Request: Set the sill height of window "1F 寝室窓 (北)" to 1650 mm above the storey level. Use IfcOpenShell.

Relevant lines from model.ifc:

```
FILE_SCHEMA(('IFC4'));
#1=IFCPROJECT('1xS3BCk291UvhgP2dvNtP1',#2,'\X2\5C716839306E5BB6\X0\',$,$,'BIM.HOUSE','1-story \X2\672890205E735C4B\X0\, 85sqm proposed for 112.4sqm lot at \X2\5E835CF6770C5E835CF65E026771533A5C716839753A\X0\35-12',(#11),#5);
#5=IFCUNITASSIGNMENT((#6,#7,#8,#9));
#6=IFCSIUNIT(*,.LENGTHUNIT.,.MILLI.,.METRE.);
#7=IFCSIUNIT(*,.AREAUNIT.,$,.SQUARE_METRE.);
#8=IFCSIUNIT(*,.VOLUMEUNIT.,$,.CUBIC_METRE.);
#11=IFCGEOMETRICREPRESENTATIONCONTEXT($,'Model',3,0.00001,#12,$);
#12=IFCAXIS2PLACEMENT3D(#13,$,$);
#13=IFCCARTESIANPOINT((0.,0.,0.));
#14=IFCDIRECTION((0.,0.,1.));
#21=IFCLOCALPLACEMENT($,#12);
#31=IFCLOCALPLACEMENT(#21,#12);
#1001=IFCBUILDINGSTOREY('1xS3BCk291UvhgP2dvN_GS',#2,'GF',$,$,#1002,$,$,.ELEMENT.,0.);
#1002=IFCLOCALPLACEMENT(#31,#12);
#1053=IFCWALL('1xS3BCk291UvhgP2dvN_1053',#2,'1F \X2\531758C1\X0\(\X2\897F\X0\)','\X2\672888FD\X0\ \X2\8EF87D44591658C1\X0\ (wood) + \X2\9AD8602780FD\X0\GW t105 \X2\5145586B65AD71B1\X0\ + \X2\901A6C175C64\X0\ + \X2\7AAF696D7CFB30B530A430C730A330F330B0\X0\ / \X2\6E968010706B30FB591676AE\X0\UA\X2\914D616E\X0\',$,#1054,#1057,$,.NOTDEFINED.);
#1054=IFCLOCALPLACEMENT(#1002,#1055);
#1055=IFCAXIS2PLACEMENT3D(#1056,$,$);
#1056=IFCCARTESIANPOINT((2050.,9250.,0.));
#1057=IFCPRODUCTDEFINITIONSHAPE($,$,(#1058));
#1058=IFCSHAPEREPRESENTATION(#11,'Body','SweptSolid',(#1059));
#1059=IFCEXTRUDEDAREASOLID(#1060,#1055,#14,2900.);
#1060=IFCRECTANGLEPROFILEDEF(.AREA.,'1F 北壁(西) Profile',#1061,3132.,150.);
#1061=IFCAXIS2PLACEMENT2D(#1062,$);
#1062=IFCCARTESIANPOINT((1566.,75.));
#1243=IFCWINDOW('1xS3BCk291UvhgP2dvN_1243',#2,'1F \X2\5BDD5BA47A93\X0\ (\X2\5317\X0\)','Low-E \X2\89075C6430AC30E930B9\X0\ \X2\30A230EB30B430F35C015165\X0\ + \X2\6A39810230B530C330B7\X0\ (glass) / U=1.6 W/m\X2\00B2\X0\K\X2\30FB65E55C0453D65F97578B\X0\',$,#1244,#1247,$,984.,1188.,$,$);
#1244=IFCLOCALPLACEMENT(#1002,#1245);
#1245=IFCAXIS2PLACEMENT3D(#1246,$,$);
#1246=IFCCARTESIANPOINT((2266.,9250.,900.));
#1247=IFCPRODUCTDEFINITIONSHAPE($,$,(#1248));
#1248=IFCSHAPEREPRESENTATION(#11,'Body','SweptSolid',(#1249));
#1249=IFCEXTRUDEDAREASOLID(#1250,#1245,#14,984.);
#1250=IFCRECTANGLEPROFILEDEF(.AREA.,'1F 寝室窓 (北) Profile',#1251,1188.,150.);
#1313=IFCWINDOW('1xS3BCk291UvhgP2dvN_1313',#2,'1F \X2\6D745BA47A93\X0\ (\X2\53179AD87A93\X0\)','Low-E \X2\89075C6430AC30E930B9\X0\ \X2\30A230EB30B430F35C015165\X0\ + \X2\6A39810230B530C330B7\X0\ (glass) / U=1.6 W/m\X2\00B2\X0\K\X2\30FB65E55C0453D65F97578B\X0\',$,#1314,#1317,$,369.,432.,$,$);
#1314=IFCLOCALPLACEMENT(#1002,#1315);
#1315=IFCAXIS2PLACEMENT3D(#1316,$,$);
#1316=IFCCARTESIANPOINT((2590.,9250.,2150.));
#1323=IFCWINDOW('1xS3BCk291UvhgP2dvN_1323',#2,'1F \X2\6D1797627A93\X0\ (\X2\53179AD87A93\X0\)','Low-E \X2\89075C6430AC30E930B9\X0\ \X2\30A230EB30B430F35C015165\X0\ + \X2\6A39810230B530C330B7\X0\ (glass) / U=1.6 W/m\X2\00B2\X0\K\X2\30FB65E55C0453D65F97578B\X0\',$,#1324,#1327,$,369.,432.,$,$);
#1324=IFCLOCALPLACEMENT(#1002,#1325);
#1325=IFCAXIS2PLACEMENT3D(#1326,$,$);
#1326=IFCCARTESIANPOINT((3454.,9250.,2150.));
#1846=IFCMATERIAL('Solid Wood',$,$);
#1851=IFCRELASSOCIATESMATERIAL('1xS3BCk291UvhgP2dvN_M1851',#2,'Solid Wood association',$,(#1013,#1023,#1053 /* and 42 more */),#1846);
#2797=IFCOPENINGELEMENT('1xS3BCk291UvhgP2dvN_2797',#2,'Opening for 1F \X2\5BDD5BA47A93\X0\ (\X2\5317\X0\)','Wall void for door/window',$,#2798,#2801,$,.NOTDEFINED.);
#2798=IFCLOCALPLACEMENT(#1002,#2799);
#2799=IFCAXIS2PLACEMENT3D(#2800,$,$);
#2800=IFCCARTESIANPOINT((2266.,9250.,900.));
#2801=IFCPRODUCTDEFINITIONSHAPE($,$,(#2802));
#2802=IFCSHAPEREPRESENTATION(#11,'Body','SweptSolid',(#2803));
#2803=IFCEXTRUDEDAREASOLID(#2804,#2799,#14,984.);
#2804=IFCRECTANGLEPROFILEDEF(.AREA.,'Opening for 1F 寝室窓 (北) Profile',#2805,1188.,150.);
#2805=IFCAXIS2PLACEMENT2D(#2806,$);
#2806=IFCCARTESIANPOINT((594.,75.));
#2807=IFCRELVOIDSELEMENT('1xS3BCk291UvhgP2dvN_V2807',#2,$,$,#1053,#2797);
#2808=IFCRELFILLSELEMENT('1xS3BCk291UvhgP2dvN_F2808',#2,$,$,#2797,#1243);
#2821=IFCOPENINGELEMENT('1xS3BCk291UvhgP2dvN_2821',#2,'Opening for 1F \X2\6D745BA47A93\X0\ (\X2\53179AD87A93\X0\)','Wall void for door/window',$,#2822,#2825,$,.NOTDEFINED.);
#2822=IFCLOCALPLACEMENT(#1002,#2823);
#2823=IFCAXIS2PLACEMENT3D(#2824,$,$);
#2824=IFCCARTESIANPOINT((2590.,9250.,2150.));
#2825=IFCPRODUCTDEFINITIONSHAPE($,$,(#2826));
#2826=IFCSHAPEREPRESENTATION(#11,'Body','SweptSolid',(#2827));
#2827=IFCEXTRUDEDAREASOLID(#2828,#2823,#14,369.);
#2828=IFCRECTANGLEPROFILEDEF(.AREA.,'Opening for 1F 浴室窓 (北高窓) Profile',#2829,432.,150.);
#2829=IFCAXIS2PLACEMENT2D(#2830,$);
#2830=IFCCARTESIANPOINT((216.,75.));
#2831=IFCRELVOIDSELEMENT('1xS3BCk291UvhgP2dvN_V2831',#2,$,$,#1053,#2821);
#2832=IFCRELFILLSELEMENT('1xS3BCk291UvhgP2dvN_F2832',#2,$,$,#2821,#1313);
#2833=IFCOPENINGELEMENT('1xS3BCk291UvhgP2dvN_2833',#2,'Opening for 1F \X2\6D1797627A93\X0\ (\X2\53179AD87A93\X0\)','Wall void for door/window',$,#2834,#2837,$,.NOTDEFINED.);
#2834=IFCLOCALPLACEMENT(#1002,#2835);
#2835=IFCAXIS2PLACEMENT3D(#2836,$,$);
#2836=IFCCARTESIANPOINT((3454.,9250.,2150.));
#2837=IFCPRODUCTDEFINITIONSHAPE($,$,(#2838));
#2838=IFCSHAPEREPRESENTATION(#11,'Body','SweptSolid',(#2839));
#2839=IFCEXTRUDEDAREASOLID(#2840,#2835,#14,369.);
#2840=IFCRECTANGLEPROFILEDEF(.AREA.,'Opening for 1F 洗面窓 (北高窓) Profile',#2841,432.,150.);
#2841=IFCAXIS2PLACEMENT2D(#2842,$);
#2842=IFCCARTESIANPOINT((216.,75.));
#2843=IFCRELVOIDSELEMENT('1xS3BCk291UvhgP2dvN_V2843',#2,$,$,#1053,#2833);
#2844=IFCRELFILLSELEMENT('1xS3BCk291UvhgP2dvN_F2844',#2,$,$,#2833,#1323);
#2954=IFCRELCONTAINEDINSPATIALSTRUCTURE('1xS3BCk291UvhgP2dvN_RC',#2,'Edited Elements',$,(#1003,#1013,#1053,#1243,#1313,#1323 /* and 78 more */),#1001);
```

```python
import numpy as np
import ifcopenshell
import ifcopenshell.api.geometry
import ifcopenshell.geom
import ifcopenshell.util.element
import ifcopenshell.util.placement
import ifcopenshell.util.shape
import ifcopenshell.util.unit

model = ifcopenshell.open("model.ifc")
unit_scale = ifcopenshell.util.unit.calculate_unit_scale(model)

window = model.by_guid("1xS3BCk291UvhgP2dvN_1243")
opening = window.FillsVoids[0].RelatingOpeningElement
storey = ifcopenshell.util.element.get_container(window, ifc_class="IfcBuildingStorey")
level = ifcopenshell.util.placement.get_local_placement(storey.ObjectPlacement)[2, 3]

# The opening's origin need not be at the sill, so measure its lowest point.
shape = ifcopenshell.geom.create_shape(ifcopenshell.geom.settings(), opening)
bottom = ifcopenshell.util.shape.get_shape_bottom_elevation(shape, shape.geometry) / unit_scale
dz = level + 1650.0 - bottom

shift = np.array([0.0, 0.0, dz])
# The window is not placed relative to its opening, so move both.
for product in (opening, window):
    matrix = ifcopenshell.util.placement.get_local_placement(product.ObjectPlacement)
    matrix[:3, 3] += shift
    ifcopenshell.api.geometry.edit_object_placement(model, product=product, matrix=matrix, is_si=False)

print(f"moved by {dz * unit_scale:+.3f} m")

model.write("model_edited.ifc")
```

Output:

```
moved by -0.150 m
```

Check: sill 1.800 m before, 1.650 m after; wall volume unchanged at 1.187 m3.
